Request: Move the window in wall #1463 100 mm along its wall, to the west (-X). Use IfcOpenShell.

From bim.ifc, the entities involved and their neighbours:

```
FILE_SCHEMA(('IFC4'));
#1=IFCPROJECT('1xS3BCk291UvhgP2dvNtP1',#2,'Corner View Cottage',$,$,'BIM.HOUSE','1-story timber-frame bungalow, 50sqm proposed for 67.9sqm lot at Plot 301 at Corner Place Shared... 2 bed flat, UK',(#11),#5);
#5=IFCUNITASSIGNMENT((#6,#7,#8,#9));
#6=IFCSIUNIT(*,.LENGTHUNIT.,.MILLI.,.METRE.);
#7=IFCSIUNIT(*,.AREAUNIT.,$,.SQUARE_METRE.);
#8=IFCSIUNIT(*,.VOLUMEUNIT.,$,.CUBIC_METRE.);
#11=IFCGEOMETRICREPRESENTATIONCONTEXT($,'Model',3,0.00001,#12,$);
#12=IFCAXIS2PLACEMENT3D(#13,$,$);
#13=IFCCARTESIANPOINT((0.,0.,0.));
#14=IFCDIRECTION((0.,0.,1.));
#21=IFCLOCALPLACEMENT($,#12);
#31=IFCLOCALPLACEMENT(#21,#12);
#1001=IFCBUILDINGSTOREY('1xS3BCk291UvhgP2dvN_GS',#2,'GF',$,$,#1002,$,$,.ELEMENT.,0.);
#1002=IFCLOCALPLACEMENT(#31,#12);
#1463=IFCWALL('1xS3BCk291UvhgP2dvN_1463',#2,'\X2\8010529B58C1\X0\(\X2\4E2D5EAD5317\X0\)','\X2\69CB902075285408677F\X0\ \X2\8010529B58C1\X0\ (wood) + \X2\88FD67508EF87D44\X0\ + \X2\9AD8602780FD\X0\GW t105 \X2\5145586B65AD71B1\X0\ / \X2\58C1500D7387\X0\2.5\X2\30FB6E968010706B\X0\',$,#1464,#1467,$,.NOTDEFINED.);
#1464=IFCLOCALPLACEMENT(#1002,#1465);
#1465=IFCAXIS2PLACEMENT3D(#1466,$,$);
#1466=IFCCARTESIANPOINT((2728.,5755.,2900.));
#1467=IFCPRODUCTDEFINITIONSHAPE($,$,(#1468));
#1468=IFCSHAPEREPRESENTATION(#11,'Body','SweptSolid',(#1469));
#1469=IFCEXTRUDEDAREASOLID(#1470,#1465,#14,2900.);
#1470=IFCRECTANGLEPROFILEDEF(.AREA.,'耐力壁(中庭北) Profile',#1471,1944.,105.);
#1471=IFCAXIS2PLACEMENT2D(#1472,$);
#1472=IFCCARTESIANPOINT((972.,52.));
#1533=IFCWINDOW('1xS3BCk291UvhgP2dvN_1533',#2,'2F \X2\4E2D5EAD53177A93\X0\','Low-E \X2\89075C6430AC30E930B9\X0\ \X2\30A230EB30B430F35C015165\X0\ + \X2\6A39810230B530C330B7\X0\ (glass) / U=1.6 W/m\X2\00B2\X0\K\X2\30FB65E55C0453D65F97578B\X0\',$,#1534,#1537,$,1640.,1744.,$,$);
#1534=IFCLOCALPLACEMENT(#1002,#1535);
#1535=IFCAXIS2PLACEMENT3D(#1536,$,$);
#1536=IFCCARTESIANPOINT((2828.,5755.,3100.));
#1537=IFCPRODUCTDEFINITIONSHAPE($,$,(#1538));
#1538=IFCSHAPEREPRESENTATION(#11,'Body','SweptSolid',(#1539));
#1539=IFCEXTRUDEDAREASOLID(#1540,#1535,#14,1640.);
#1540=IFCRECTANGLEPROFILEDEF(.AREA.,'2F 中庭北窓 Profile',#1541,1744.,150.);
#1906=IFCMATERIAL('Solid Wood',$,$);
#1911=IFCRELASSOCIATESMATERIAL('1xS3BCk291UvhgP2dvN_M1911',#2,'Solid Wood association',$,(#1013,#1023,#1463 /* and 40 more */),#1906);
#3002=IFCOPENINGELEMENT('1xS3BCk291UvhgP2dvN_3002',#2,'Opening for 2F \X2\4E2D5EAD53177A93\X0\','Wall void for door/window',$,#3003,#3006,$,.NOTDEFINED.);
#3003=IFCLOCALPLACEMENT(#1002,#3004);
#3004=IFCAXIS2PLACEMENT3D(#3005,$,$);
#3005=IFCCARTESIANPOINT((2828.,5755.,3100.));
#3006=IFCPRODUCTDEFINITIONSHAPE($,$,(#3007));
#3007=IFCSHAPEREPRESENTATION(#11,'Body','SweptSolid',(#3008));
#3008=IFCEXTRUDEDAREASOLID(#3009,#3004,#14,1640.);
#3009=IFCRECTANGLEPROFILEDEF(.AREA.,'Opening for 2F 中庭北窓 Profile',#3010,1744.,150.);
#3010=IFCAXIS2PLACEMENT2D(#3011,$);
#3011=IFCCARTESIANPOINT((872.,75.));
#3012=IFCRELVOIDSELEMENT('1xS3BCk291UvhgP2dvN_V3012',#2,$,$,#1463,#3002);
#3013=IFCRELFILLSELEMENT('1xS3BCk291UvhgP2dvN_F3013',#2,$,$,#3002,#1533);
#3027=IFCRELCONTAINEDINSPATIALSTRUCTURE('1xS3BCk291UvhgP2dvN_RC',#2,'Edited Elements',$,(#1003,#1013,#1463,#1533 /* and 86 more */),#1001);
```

```python
import ifcopenshell
import ifcopenshell.api.geometry
import ifcopenshell.util.placement

model = ifcopenshell.open("bim.ifc")

window = model.by_id(1533)
opening = window.FillsVoids[0].RelatingOpeningElement
wall = opening.VoidsElements[0].RelatingBuildingElement

wall_matrix = ifcopenshell.util.placement.get_local_placement(wall.ObjectPlacement)
shift = wall_matrix[:3, 0] * -100.0
before = ifcopenshell.util.placement.get_local_placement(window.ObjectPlacement)[:3, 3].copy()

# The window is not placed relative to its opening, so move both.
for product in (opening, window):
    matrix = ifcopenshell.util.placement.get_local_placement(product.ObjectPlacement)
    matrix[:3, 3] += shift
    ifcopenshell.api.geometry.edit_object_placement(model, product=product, matrix=matrix, is_si=False)

after = ifcopenshell.util.placement.get_local_placement(window.ObjectPlacement)[:3, 3]
print("window moved by", (after - before).round(3) + 0.0)

model.write("bim_updated.ifc")
```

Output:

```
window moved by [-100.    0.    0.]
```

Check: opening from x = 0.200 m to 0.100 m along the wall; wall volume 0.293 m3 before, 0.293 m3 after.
